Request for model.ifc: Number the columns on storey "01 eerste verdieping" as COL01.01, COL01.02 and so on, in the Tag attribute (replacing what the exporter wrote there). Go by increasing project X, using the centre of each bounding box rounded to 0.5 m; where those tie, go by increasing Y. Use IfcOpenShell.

First a look at what the model holds.

```python
import ifcopenshell
import ifcopenshell.util.element
import ifcopenshell.util.placement

model = ifcopenshell.open("model.ifc")
print(model.schema)
storey = next(s for s in model.by_type("IfcBuildingStorey") if s.Name == "01 eerste verdieping")
columns = [e for e in ifcopenshell.util.element.get_decomposition(storey) if e.is_a("IfcColumn")]
for e in sorted(columns, key=lambda e: e.id()):
    origin = ifcopenshell.util.placement.get_local_placement(e.ObjectPlacement)[:3, 3]
    print(e.id(), e.Tag, e.Name, origin.round(2) + 0.0, sep=" | ")
```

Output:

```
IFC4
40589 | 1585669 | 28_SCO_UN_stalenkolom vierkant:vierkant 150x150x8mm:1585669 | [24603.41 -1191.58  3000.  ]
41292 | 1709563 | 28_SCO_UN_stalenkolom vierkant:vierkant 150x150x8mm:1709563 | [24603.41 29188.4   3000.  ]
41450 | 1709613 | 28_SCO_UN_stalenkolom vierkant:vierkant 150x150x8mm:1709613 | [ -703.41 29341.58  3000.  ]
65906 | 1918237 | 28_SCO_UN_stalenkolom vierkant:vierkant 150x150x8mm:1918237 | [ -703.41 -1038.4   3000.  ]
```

```python
import ifcopenshell
import ifcopenshell.geom
import ifcopenshell.util.element
import ifcopenshell.util.shape

model = ifcopenshell.open("model.ifc")
settings = ifcopenshell.geom.settings()
settings.set("use-world-coords", True)


def centre(element):
    shape = ifcopenshell.geom.create_shape(settings, element)
    return ifcopenshell.util.shape.get_bbox_centroid(shape.geometry)


storey = next(s for s in model.by_type("IfcBuildingStorey") if s.Name == "01 eerste verdieping")
columns = [e for e in ifcopenshell.util.element.get_decomposition(storey) if e.is_a("IfcColumn")]

# Insertion points can sit at a corner or the storey origin, so sort by the geometry (in metres).
centres = {e: centre(e) for e in columns}
columns.sort(key=lambda e: (round(centres[e][0] / 0.5), centres[e][1]))

for i, e in enumerate(columns, start=1):
    number = f"COL01.{i:02d}"
    e.Tag = number
    print(e.id(), number)

model.write("model_rev.ifc")
```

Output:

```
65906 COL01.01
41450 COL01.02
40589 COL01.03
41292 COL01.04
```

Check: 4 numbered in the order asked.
